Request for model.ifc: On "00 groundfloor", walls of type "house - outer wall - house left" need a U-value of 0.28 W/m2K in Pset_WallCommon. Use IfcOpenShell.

First a look at what the model holds.

```python
import ifcopenshell
import ifcopenshell.util.element

model = ifcopenshell.open("model.ifc")
print(model.schema)
storey = next(s for s in model.by_type("IfcBuildingStorey") if s.Name == "00 groundfloor")
walls = [e for e in ifcopenshell.util.element.get_decomposition(storey) if e.is_a("IfcWall")]
seen = {}
for e in walls:
    element_type = ifcopenshell.util.element.get_type(e)
    key = (element_type.Name if element_type != e and element_type else None, ifcopenshell.util.element.get_pset(e, "Pset_WallCommon", "ThermalTransmittance"))
    seen[key] = seen.get(key, 0) + 1
for (name, value), count in sorted(seen.items(), key=str):
    print(count, "x", name, "|", value)
```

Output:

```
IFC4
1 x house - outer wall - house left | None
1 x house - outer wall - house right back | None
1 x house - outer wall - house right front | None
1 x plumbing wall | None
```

```python
import ifcopenshell
import ifcopenshell.api.pset
import ifcopenshell.util.element

model = ifcopenshell.open("model.ifc")

storey = next(s for s in model.by_type("IfcBuildingStorey") if s.Name == "00 groundfloor")
walls = [e for e in ifcopenshell.util.element.get_decomposition(storey) if e.is_a("IfcWall")]

count = 0
for e in walls:
    element_type = ifcopenshell.util.element.get_type(e)
    if element_type in (None, e) or element_type.Name != "house - outer wall - house left":
        continue
    # add_pset returns the element's existing set when there is one.
    pset = ifcopenshell.api.pset.add_pset(model, product=e, name="Pset_WallCommon")
    ifcopenshell.api.pset.edit_pset(model, pset=pset, properties={"ThermalTransmittance": 0.28})
    count += 1

print(count, "walls updated")

model.write("model_v2.ifc")
```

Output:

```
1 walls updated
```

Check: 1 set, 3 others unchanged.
